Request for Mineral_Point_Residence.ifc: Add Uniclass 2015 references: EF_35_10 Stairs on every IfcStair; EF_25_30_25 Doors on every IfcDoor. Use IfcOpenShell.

First a look at what the model holds.

```python
import ifcopenshell

model = ifcopenshell.open("Mineral_Point_Residence.ifc")
print(model.schema)
print("classifications:", [c.Name for c in model.by_type("IfcClassification")])
for ifc_class in ("IfcDoor", "IfcRoof", "IfcStair", "IfcWall", "IfcWindow"):
    print(ifc_class, len(model.by_type(ifc_class)))
```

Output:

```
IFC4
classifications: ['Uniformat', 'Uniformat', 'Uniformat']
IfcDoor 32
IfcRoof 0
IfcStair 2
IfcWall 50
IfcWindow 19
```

```python
import ifcopenshell
import ifcopenshell.api.classification

model = ifcopenshell.open("Mineral_Point_Residence.ifc")

system = ifcopenshell.api.classification.add_classification(model, classification="Uniclass 2015")

codes = {
    "IfcStair": ("EF_35_10", "Stairs"),
    "IfcDoor": ("EF_25_30_25", "Doors"),
}
for ifc_class, (code, name) in codes.items():
    products = model.by_type(ifc_class)
    ifcopenshell.api.classification.add_reference(
        model, products=products, classification=system, identification=code, name=name
    )
    print(code, len(products))

model.write("Mineral_Point_Residence_v2.ifc")
```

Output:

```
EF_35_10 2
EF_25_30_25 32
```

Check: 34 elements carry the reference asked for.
